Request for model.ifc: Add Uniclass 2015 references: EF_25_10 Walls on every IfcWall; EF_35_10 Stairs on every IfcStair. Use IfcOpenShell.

First a look at what the model holds.

```python
import ifcopenshell

model = ifcopenshell.open("model.ifc")
print(model.schema)
print("classifications:", [c.Name for c in model.by_type("IfcClassification")])
for ifc_class in ("IfcDoor", "IfcRoof", "IfcStair", "IfcWall", "IfcWindow"):
    print(ifc_class, len(model.by_type(ifc_class)))
```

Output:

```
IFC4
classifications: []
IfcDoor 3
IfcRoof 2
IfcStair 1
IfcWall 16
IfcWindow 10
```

```python
import ifcopenshell
import ifcopenshell.api.classification

model = ifcopenshell.open("model.ifc")

system = ifcopenshell.api.classification.add_classification(model, classification="Uniclass 2015")

codes = {
    "IfcWall": ("EF_25_10", "Walls"),
    "IfcStair": ("EF_35_10", "Stairs"),
}
for ifc_class, (code, name) in codes.items():
    products = model.by_type(ifc_class)
    ifcopenshell.api.classification.add_reference(
        model, products=products, classification=system, identification=code, name=name
    )
    print(code, len(products))

model.write("model_updated.ifc")
```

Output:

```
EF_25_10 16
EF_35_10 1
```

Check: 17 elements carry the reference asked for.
